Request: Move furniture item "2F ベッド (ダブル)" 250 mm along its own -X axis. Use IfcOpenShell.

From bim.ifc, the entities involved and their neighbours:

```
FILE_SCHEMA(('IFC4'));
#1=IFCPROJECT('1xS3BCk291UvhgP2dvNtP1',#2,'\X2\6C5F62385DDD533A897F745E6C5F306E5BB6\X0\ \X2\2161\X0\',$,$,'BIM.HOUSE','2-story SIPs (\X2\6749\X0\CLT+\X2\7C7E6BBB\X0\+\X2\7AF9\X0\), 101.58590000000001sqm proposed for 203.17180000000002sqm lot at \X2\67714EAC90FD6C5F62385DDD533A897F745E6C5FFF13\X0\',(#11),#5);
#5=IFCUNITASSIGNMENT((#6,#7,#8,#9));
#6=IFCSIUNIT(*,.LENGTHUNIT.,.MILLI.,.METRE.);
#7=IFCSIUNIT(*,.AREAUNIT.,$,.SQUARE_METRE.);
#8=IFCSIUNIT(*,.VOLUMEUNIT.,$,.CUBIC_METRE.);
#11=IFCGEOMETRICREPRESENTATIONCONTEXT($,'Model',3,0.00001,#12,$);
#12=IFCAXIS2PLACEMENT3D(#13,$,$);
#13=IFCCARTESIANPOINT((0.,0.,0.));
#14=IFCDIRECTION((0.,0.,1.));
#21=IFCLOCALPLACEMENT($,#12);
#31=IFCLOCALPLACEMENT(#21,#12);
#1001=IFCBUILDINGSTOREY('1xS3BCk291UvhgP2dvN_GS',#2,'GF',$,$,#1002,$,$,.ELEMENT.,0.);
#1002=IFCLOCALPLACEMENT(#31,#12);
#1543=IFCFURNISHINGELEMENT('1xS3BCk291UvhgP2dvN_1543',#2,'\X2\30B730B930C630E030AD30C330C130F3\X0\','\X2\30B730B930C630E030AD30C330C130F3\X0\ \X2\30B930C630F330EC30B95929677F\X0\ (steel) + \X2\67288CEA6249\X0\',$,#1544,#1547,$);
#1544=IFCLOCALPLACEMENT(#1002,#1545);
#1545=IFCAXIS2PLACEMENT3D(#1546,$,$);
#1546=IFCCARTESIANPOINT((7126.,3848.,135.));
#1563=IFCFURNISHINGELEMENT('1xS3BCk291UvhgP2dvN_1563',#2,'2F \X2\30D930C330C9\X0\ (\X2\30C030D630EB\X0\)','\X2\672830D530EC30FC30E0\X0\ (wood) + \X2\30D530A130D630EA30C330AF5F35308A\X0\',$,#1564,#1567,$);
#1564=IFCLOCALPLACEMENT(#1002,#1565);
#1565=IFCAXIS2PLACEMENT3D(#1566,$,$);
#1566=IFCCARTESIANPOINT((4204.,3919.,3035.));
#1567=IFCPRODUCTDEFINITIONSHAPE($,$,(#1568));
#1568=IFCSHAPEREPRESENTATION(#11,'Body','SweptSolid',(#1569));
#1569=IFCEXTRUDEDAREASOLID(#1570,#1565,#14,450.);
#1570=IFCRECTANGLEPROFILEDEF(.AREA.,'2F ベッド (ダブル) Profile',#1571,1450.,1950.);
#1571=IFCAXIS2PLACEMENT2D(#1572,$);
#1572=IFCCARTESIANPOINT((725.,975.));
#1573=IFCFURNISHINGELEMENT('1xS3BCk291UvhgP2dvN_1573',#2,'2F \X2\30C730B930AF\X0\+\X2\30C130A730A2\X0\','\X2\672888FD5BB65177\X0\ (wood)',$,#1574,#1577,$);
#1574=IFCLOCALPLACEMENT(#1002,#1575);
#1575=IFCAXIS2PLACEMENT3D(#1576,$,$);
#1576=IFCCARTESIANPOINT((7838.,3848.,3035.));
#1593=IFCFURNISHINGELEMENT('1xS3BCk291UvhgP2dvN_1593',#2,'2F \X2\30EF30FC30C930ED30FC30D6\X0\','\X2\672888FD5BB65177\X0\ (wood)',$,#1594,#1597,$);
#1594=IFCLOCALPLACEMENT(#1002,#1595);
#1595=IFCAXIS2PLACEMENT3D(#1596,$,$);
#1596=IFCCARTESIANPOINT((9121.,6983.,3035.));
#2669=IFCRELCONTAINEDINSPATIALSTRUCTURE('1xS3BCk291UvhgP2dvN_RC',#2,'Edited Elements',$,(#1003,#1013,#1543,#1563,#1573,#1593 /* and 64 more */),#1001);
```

```python
import ifcopenshell
import ifcopenshell.api.geometry
import ifcopenshell.util.placement
import ifcopenshell.util.unit

model = ifcopenshell.open("bim.ifc")
unit_scale = ifcopenshell.util.unit.calculate_unit_scale(model)

item = model.by_guid("1xS3BCk291UvhgP2dvN_1563")
matrix = ifcopenshell.util.placement.get_local_placement(item.ObjectPlacement)
matrix[:3, 3] -= matrix[:3, 0] * 0.25 / unit_scale
ifcopenshell.api.geometry.edit_object_placement(model, product=item, matrix=matrix, is_si=False)

print(ifcopenshell.util.placement.get_local_placement(item.ObjectPlacement).round(3) + 0.0)

model.write("bim_updated.ifc")
```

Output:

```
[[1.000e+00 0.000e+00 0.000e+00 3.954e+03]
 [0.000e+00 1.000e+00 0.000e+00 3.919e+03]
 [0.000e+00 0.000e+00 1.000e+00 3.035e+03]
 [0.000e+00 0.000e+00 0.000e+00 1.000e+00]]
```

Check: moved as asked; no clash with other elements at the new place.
